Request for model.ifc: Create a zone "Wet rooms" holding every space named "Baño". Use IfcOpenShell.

First a look at what the model holds.

```python
import ifcopenshell

model = ifcopenshell.open("model.ifc")
print(model.schema)
seen = {}
for space in model.by_type("IfcSpace"):
    seen[space.LongName] = seen.get(space.LongName, 0) + 1
for name, count in sorted(seen.items(), key=str):
    print(count, "x", name)
print("zones:", [z.Name for z in model.by_type("IfcZone")][:20])
```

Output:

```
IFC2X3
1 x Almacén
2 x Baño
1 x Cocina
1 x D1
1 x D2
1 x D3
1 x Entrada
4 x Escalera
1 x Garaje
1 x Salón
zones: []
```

```python
import ifcopenshell
import ifcopenshell.api.group
import ifcopenshell.api.root

model = ifcopenshell.open("model.ifc")

names = {"Baño"}
spaces = [s for s in model.by_type("IfcSpace") if s.LongName in names]

zone = ifcopenshell.api.root.create_entity(model, ifc_class="IfcZone", name="Wet rooms")
ifcopenshell.api.group.assign_group(model, products=spaces, group=zone)
print(len(spaces), "spaces in", zone.Name)

model.write("model_rev.ifc")
```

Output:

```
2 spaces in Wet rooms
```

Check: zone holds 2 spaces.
